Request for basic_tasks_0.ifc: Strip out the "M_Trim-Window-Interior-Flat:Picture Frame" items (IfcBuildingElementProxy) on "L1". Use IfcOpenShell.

First a look at what the model holds.

```python
import ifcopenshell
import ifcopenshell.util.element

model = ifcopenshell.open("basic_tasks_0.ifc")
print(model.schema)
storey = next(s for s in model.by_type("IfcBuildingStorey") if s.Name == "L1")
proxies = [e for e in ifcopenshell.util.element.get_decomposition(storey) if e.is_a("IfcBuildingElementProxy")]
seen = {}
for e in proxies:
    element_type = ifcopenshell.util.element.get_type(e)
    name = element_type.Name if element_type not in (None, e) else None
    seen[name] = seen.get(name, 0) + 1
for name, count in sorted(seen.items(), key=str):
    print(count, "x", name)
```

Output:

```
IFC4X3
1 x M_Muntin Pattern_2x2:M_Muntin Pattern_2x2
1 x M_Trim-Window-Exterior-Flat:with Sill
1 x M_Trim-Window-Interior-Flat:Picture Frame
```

```python
import ifcopenshell
import ifcopenshell.api.root
import ifcopenshell.util.element

model = ifcopenshell.open("basic_tasks_0.ifc")

storey = next(s for s in model.by_type("IfcBuildingStorey") if s.Name == "L1")
proxies = [e for e in ifcopenshell.util.element.get_decomposition(storey) if e.is_a("IfcBuildingElementProxy")]
targets = [e for e in proxies if (t := ifcopenshell.util.element.get_type(e)) not in (None, e) and t.Name == "M_Trim-Window-Interior-Flat:Picture Frame"]

for e in targets:
    ifcopenshell.api.root.remove_product(model, product=e)
print(len(targets), "removed")

model.write("basic_tasks_0-out.ifc")
```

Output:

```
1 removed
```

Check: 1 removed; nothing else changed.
